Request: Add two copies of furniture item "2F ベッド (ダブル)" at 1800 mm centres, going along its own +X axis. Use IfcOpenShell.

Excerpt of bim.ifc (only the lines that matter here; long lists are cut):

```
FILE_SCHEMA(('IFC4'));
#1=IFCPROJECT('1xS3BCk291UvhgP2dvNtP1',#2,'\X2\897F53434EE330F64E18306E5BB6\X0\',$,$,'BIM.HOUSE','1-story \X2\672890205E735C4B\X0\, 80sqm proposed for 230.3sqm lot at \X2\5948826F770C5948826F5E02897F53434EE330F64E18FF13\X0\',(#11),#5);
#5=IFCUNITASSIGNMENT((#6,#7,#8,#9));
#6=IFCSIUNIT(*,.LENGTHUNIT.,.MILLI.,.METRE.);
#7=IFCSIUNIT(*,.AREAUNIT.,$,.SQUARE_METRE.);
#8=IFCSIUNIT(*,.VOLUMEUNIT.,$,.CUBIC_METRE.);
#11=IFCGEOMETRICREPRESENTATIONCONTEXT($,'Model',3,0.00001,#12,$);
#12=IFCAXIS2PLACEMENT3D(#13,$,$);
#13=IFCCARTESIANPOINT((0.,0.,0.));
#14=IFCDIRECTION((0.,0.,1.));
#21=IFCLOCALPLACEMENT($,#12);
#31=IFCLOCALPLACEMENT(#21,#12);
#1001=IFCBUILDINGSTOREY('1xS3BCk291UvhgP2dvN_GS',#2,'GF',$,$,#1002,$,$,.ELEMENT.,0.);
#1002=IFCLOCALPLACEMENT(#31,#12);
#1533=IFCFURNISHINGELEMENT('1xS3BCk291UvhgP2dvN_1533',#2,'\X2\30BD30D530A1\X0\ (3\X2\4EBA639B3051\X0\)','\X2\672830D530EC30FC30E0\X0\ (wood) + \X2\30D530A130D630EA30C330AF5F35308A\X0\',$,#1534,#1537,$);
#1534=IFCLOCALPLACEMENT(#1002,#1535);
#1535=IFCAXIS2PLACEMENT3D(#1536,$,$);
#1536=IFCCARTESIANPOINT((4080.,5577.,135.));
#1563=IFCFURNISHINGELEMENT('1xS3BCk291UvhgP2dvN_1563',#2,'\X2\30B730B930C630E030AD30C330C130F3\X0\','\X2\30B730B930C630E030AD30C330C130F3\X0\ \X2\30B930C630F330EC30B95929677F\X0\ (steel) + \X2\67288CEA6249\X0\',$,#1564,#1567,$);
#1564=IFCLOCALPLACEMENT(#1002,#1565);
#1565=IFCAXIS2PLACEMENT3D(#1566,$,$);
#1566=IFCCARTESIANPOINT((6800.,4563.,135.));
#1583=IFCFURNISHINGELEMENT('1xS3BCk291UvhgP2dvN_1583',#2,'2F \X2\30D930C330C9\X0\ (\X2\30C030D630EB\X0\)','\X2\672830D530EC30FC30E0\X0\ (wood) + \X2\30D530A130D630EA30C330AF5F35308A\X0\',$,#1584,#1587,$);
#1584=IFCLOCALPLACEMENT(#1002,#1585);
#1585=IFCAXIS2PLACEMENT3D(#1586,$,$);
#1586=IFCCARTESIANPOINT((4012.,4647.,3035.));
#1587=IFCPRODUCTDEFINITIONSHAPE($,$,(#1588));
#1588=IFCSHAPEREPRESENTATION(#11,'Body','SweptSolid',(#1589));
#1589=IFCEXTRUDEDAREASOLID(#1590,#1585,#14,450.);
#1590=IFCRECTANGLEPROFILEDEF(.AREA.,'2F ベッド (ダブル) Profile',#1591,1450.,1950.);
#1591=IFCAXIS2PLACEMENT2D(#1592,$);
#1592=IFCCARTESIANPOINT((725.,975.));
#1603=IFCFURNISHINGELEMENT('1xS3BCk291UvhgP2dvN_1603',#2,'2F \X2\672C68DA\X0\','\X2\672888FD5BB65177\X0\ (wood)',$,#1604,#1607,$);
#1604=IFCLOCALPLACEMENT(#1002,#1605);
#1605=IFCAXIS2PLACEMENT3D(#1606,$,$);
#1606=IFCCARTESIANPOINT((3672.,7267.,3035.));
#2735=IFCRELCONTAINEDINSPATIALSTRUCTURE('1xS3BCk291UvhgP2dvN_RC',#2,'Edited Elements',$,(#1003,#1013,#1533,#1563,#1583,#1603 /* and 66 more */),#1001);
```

```python
import ifcopenshell
import ifcopenshell.api.geometry
import ifcopenshell.api.root
import ifcopenshell.util.element
import ifcopenshell.util.placement

model = ifcopenshell.open("bim.ifc")


def reuse_history(source, copy):
    """copy_class also copies each property set's owner history, people and application; keep the originals."""
    for rel in copy.IsDefinedBy:
        if rel.is_a("IfcRelDefinesByProperties") and (history := rel.RelatingPropertyDefinition.OwnerHistory):
            rel.RelatingPropertyDefinition.OwnerHistory = source.OwnerHistory
            ifcopenshell.util.element.remove_deep2(model, history)


source = model.by_guid("1xS3BCk291UvhgP2dvN_1583")
base = ifcopenshell.util.placement.get_local_placement(source.ObjectPlacement)
step = base[:3, 0] * 1800.0

for i in range(1, 3):
    copy = ifcopenshell.api.root.copy_class(model, product=source)
    copy.Representation = ifcopenshell.util.element.copy_deep(
        model, source.Representation, exclude=["IfcGeometricRepresentationContext", "IfcRepresentationMap"]
    )
    reuse_history(source, copy)
    matrix = base.copy()
    matrix[:3, 3] += i * step
    print("added at", matrix[:3, 3].round(3) + 0.0)
    ifcopenshell.api.geometry.edit_object_placement(model, product=copy, matrix=matrix, is_si=False)

model.write("bim-out.ifc")
```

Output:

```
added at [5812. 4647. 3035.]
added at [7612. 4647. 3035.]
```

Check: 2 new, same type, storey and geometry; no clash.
